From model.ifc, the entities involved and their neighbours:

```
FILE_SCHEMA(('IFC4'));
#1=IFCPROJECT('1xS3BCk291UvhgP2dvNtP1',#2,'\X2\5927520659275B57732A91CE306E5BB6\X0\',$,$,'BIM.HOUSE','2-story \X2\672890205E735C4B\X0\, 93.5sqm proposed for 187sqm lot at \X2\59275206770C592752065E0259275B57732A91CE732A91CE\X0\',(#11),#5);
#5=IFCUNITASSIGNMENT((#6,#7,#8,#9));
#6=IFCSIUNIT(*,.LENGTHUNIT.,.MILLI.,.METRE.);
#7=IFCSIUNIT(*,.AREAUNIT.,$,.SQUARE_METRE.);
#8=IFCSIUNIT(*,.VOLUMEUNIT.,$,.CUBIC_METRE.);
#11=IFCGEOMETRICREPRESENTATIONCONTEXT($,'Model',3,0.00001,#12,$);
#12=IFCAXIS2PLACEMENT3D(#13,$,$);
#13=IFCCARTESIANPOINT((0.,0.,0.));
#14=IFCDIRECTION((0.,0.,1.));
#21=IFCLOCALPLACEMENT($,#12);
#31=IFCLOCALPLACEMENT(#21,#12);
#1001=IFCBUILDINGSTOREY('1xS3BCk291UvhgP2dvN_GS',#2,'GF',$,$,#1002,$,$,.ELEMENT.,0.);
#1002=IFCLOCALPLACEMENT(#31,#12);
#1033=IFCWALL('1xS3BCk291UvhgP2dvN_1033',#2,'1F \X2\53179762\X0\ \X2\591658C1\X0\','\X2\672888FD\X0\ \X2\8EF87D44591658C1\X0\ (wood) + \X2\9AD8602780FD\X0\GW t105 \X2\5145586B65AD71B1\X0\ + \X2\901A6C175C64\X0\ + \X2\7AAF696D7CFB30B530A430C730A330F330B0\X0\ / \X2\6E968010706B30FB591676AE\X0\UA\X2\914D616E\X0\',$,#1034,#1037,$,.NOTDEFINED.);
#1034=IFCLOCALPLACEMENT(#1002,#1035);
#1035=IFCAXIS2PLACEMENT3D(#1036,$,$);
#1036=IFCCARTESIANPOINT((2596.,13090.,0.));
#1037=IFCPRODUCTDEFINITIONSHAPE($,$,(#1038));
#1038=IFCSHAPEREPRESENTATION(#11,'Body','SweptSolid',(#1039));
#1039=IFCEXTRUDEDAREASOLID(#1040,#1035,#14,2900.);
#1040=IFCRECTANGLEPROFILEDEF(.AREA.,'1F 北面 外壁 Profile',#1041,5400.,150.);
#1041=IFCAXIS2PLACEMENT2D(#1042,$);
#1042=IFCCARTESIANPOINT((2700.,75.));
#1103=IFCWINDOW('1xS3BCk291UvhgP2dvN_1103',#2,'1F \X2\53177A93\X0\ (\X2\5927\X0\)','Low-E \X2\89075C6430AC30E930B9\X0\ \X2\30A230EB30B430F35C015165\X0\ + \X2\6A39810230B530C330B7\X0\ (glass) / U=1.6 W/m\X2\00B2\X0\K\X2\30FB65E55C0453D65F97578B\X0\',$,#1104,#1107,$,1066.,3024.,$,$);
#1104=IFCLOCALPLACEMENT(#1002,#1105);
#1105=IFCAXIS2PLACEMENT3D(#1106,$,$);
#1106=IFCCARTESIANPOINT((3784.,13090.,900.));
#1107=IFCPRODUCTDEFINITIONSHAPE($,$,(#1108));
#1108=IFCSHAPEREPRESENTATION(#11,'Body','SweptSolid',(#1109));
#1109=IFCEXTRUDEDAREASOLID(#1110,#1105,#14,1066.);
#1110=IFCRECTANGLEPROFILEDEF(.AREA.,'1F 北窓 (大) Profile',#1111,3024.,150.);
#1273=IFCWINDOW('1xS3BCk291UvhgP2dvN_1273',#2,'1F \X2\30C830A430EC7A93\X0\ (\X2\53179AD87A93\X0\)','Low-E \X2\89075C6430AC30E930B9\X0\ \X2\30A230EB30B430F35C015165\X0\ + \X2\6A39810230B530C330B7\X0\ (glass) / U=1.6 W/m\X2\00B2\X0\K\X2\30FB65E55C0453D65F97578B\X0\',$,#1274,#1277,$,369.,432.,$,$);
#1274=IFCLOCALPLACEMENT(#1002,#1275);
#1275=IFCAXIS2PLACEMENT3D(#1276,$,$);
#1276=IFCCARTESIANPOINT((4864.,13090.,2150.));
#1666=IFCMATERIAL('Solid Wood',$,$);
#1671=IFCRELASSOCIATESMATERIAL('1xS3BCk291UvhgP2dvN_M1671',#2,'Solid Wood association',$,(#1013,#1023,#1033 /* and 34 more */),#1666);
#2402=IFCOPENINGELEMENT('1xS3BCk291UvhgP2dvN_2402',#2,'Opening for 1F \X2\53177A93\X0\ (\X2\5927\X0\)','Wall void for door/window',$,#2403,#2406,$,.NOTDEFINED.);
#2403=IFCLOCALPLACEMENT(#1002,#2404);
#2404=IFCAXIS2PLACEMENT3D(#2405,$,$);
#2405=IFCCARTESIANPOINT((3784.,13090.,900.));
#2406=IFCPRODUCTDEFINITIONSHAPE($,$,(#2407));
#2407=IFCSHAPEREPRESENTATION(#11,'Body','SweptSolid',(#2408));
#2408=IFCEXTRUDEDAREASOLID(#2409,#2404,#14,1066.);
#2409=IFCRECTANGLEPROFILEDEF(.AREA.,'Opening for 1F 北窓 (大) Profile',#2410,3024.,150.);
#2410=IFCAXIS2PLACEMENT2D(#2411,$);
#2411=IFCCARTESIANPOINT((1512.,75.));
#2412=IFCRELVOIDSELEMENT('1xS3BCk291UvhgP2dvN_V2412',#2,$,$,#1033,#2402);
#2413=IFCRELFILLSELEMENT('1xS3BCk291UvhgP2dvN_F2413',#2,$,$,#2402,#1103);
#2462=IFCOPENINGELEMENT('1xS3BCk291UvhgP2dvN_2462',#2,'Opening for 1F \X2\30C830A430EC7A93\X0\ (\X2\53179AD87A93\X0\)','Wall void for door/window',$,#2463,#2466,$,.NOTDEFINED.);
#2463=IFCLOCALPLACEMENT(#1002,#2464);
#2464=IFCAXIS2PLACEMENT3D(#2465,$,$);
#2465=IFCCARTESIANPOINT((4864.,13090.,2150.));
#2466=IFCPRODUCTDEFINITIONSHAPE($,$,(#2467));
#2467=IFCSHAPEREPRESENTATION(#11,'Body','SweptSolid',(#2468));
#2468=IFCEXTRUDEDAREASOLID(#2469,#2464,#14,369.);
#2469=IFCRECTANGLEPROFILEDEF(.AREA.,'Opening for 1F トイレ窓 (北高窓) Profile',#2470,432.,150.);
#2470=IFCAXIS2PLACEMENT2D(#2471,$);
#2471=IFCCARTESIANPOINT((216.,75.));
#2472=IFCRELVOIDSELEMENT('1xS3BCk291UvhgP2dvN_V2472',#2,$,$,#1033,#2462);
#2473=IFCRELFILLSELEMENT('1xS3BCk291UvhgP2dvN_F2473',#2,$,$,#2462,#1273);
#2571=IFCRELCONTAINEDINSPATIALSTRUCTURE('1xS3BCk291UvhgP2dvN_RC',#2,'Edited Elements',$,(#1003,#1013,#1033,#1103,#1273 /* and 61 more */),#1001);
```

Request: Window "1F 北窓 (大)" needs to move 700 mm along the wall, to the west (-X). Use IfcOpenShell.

```python
import ifcopenshell
import ifcopenshell.api.geometry
import ifcopenshell.util.placement
import ifcopenshell.util.unit

model = ifcopenshell.open("model.ifc")
unit_scale = ifcopenshell.util.unit.calculate_unit_scale(model)

window = model.by_guid("1xS3BCk291UvhgP2dvN_1103")
opening = window.FillsVoids[0].RelatingOpeningElement
wall = opening.VoidsElements[0].RelatingBuildingElement

wall_matrix = ifcopenshell.util.placement.get_local_placement(wall.ObjectPlacement)
shift = wall_matrix[:3, 0] * -0.7 / unit_scale
before = ifcopenshell.util.placement.get_local_placement(window.ObjectPlacement)[:3, 3].copy()

# The window is not placed relative to its opening, so move both.
for product in (opening, window):
    matrix = ifcopenshell.util.placement.get_local_placement(product.ObjectPlacement)
    matrix[:3, 3] += shift
    ifcopenshell.api.geometry.edit_object_placement(model, product=product, matrix=matrix, is_si=False)

after = ifcopenshell.util.placement.get_local_placement(window.ObjectPlacement)[:3, 3]
print("window moved by", (after - before).round(3) + 0.0)

model.write("model_v2.ifc")
```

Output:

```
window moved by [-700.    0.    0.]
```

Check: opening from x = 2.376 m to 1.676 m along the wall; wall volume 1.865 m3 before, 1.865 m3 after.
